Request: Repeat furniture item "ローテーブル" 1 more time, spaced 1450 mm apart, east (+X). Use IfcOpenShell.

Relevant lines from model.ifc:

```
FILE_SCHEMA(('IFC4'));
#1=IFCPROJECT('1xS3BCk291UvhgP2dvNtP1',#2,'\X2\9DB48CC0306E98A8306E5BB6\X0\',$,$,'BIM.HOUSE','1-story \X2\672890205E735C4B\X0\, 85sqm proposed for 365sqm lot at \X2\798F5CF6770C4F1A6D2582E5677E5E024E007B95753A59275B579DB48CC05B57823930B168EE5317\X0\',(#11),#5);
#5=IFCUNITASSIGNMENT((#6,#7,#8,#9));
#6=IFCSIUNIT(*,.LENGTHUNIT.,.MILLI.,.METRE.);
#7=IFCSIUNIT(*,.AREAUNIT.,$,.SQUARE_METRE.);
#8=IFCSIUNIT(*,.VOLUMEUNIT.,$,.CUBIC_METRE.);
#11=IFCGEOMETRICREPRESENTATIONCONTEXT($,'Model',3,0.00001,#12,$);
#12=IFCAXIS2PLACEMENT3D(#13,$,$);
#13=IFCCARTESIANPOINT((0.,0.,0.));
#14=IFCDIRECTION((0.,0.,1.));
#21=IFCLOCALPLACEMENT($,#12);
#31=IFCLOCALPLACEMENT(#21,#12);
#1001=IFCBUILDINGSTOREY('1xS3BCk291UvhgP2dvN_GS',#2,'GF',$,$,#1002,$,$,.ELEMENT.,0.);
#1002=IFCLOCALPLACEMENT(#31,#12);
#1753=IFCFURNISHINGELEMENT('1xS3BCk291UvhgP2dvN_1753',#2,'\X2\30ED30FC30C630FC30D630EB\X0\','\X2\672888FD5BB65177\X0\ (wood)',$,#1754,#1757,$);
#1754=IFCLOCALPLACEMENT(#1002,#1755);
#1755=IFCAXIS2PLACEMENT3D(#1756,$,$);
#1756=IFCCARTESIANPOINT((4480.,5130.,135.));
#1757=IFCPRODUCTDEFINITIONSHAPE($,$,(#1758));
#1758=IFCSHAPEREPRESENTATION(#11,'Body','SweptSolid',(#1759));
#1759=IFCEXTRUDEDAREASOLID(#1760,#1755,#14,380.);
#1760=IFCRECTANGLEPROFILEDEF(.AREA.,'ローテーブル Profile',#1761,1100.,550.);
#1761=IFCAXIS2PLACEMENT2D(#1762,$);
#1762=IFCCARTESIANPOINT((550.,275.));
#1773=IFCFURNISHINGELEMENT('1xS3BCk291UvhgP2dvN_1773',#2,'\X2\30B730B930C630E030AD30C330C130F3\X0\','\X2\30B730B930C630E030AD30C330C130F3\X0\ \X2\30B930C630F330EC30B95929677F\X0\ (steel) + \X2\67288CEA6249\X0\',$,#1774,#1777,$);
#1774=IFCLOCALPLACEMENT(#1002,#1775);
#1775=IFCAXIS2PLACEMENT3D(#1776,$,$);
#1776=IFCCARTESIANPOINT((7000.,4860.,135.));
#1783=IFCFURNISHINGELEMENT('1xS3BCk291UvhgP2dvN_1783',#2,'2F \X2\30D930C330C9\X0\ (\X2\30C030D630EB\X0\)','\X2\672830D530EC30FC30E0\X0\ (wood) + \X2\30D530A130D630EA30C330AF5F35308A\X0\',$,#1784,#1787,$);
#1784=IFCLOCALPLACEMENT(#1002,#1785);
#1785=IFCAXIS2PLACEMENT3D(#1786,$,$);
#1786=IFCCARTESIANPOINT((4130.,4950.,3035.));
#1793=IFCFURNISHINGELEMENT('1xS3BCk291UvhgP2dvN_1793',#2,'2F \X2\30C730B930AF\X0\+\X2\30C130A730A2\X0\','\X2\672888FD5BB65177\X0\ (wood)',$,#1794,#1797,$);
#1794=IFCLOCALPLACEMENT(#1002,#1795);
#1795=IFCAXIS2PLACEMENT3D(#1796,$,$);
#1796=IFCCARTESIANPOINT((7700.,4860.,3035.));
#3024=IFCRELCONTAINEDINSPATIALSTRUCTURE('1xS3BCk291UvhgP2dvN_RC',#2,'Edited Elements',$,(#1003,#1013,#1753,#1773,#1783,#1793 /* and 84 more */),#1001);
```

```python
import numpy as np
import ifcopenshell
import ifcopenshell.api.geometry
import ifcopenshell.api.root
import ifcopenshell.util.element
import ifcopenshell.util.placement

model = ifcopenshell.open("model.ifc")


def reuse_history(source, copy):
    """copy_class also copies each property set's owner history, people and application; keep the originals."""
    for rel in copy.IsDefinedBy:
        if rel.is_a("IfcRelDefinesByProperties") and (history := rel.RelatingPropertyDefinition.OwnerHistory):
            rel.RelatingPropertyDefinition.OwnerHistory = source.OwnerHistory
            ifcopenshell.util.element.remove_deep2(model, history)


source = model.by_guid("1xS3BCk291UvhgP2dvN_1753")
base = ifcopenshell.util.placement.get_local_placement(source.ObjectPlacement)
step = np.array([1.0, 0.0, 0.0]) * 1450.0

for i in range(1, 2):
    copy = ifcopenshell.api.root.copy_class(model, product=source)
    copy.Representation = ifcopenshell.util.element.copy_deep(
        model, source.Representation, exclude=["IfcGeometricRepresentationContext", "IfcRepresentationMap"]
    )
    reuse_history(source, copy)
    matrix = base.copy()
    matrix[:3, 3] += i * step
    print("added at", matrix[:3, 3].round(3) + 0.0)
    ifcopenshell.api.geometry.edit_object_placement(model, product=copy, matrix=matrix, is_si=False)

model.write("model_rev.ifc")
```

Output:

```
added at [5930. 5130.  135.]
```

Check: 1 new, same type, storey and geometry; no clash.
